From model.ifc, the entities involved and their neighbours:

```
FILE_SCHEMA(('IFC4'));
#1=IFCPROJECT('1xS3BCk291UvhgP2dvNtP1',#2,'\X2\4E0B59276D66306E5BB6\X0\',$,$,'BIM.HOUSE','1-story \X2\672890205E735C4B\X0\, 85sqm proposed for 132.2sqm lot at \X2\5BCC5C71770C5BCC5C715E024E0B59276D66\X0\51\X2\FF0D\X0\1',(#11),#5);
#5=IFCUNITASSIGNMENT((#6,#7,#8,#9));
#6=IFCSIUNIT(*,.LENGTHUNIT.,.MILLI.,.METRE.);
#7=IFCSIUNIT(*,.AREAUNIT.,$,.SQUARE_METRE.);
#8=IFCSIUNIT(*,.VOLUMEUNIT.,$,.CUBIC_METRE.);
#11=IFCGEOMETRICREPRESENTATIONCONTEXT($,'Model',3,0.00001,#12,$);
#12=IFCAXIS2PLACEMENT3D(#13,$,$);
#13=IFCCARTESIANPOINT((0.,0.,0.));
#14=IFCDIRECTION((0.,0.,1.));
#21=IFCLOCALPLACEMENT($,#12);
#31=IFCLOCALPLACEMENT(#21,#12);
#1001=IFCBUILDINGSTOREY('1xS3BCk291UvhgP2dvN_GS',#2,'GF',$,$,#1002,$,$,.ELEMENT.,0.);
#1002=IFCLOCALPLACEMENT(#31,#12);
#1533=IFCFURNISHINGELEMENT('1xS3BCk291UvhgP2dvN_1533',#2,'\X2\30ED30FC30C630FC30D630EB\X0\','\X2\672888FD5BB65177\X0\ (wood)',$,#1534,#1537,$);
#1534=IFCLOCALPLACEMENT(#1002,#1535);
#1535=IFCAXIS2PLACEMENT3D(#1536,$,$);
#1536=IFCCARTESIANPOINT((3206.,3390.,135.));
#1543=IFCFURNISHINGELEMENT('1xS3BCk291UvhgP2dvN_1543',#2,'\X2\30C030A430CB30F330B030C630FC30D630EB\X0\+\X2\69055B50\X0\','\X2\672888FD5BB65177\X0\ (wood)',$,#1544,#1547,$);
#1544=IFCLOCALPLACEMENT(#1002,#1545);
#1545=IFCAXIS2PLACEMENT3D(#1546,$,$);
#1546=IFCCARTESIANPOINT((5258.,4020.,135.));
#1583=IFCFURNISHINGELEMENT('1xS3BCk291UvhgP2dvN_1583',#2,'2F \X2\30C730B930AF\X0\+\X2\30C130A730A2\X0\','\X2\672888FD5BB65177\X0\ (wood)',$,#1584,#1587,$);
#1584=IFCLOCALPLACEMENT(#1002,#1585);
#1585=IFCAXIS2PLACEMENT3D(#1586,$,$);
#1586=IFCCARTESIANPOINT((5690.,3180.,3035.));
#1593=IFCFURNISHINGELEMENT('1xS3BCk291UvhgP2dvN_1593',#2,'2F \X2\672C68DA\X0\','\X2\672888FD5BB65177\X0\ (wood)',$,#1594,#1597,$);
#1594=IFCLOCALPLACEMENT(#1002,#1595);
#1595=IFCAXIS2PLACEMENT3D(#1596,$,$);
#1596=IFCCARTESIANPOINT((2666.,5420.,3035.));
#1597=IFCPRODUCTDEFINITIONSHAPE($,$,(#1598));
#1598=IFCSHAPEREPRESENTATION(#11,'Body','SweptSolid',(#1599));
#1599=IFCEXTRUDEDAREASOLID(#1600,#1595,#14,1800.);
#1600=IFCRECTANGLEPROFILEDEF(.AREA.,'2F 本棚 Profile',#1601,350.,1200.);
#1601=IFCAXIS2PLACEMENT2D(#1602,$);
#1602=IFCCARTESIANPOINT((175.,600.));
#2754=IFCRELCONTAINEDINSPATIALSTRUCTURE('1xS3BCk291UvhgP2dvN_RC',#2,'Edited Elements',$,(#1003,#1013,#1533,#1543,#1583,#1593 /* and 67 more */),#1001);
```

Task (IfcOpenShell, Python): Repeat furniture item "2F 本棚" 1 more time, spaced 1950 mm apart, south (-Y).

```python
import numpy as np
import ifcopenshell
import ifcopenshell.api.geometry
import ifcopenshell.api.root
import ifcopenshell.util.element
import ifcopenshell.util.placement
import ifcopenshell.util.unit

model = ifcopenshell.open("model.ifc")
unit_scale = ifcopenshell.util.unit.calculate_unit_scale(model)


def reuse_history(source, copy):
    """copy_class also copies each property set's owner history, people and application; keep the originals."""
    for rel in copy.IsDefinedBy:
        if rel.is_a("IfcRelDefinesByProperties") and (history := rel.RelatingPropertyDefinition.OwnerHistory):
            rel.RelatingPropertyDefinition.OwnerHistory = source.OwnerHistory
            ifcopenshell.util.element.remove_deep2(model, history)


source = model.by_id(1593)
base = ifcopenshell.util.placement.get_local_placement(source.ObjectPlacement)
step = np.array([0.0, -1.0, 0.0]) * 1.95 / unit_scale

for i in range(1, 2):
    copy = ifcopenshell.api.root.copy_class(model, product=source)
    copy.Representation = ifcopenshell.util.element.copy_deep(
        model, source.Representation, exclude=["IfcGeometricRepresentationContext", "IfcRepresentationMap"]
    )
    reuse_history(source, copy)
    matrix = base.copy()
    matrix[:3, 3] += i * step
    print("added at", matrix[:3, 3].round(3) + 0.0)
    ifcopenshell.api.geometry.edit_object_placement(model, product=copy, matrix=matrix, is_si=False)

model.write("model_v2.ifc")
```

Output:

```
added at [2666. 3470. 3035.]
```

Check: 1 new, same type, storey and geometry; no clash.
